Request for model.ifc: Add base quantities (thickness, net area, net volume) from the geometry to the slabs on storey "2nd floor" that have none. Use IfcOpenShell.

First a look at what the model holds.

```python
import ifcopenshell
import ifcopenshell.util.element
import ifcopenshell.util.unit

model = ifcopenshell.open("model.ifc")
print(model.schema)
for unit_type in ("LENGTHUNIT", "AREAUNIT", "VOLUMEUNIT"):
    print(unit_type, ifcopenshell.util.unit.calculate_unit_scale(model, unit_type))
storey = next(s for s in model.by_type("IfcBuildingStorey") if s.Name == "2nd floor")
slabs = [e for e in ifcopenshell.util.element.get_decomposition(storey) if e.is_a("IfcSlab")]
for e in sorted(slabs, key=lambda e: e.id()):
    print(e.id(), e.is_a(), e.Name, list(ifcopenshell.util.element.get_psets(e, qtos_only=True)), sep=" | ")
```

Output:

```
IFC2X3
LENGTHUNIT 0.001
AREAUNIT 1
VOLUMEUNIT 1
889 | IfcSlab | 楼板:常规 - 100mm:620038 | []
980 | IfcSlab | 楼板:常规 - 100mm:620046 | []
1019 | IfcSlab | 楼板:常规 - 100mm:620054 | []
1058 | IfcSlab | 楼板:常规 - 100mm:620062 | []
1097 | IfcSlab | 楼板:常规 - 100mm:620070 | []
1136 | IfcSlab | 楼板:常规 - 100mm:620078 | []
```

```python
import ifcopenshell
import ifcopenshell.api.pset
import ifcopenshell.geom
import ifcopenshell.util.element
import ifcopenshell.util.shape
import ifcopenshell.util.unit

model = ifcopenshell.open("model.ifc")
unit_scale = ifcopenshell.util.unit.calculate_unit_scale(model)
area_scale = ifcopenshell.util.unit.calculate_unit_scale(model, "AREAUNIT")
volume_scale = ifcopenshell.util.unit.calculate_unit_scale(model, "VOLUMEUNIT")
settings = ifcopenshell.geom.settings()

storey = next(s for s in model.by_type("IfcBuildingStorey") if s.Name == "2nd floor")
slabs = [e for e in ifcopenshell.util.element.get_decomposition(storey) if e.is_a("IfcSlab")]

for e in sorted(slabs, key=lambda e: e.id()):
    if ifcopenshell.util.element.get_psets(e, qtos_only=True, should_inherit=False):
        continue
    # Geometry comes back in metres, in the element's own axes.
    shape = ifcopenshell.geom.create_shape(settings, e)
    values = {
        "Width": ifcopenshell.util.shape.get_z(shape.geometry) / unit_scale,
        "NetArea": ifcopenshell.util.shape.get_footprint_area(shape.geometry) / area_scale,
        "NetVolume": ifcopenshell.util.shape.get_volume(shape.geometry) / volume_scale,
    }
    qto = ifcopenshell.api.pset.add_qto(model, product=e, name="BaseQuantities")
    ifcopenshell.api.pset.edit_qto(model, qto=qto, properties=values)
    print(e.id(), {k: round(v, 3) for k, v in values.items()})

model.write("model-out.ifc")
```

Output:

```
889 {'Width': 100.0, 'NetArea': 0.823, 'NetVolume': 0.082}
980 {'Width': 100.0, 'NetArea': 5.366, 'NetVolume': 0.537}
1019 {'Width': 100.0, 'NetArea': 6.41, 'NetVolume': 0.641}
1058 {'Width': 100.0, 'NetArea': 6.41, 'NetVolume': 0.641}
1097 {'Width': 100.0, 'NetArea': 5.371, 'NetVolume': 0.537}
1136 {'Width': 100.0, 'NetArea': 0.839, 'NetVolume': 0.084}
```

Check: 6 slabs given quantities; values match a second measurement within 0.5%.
